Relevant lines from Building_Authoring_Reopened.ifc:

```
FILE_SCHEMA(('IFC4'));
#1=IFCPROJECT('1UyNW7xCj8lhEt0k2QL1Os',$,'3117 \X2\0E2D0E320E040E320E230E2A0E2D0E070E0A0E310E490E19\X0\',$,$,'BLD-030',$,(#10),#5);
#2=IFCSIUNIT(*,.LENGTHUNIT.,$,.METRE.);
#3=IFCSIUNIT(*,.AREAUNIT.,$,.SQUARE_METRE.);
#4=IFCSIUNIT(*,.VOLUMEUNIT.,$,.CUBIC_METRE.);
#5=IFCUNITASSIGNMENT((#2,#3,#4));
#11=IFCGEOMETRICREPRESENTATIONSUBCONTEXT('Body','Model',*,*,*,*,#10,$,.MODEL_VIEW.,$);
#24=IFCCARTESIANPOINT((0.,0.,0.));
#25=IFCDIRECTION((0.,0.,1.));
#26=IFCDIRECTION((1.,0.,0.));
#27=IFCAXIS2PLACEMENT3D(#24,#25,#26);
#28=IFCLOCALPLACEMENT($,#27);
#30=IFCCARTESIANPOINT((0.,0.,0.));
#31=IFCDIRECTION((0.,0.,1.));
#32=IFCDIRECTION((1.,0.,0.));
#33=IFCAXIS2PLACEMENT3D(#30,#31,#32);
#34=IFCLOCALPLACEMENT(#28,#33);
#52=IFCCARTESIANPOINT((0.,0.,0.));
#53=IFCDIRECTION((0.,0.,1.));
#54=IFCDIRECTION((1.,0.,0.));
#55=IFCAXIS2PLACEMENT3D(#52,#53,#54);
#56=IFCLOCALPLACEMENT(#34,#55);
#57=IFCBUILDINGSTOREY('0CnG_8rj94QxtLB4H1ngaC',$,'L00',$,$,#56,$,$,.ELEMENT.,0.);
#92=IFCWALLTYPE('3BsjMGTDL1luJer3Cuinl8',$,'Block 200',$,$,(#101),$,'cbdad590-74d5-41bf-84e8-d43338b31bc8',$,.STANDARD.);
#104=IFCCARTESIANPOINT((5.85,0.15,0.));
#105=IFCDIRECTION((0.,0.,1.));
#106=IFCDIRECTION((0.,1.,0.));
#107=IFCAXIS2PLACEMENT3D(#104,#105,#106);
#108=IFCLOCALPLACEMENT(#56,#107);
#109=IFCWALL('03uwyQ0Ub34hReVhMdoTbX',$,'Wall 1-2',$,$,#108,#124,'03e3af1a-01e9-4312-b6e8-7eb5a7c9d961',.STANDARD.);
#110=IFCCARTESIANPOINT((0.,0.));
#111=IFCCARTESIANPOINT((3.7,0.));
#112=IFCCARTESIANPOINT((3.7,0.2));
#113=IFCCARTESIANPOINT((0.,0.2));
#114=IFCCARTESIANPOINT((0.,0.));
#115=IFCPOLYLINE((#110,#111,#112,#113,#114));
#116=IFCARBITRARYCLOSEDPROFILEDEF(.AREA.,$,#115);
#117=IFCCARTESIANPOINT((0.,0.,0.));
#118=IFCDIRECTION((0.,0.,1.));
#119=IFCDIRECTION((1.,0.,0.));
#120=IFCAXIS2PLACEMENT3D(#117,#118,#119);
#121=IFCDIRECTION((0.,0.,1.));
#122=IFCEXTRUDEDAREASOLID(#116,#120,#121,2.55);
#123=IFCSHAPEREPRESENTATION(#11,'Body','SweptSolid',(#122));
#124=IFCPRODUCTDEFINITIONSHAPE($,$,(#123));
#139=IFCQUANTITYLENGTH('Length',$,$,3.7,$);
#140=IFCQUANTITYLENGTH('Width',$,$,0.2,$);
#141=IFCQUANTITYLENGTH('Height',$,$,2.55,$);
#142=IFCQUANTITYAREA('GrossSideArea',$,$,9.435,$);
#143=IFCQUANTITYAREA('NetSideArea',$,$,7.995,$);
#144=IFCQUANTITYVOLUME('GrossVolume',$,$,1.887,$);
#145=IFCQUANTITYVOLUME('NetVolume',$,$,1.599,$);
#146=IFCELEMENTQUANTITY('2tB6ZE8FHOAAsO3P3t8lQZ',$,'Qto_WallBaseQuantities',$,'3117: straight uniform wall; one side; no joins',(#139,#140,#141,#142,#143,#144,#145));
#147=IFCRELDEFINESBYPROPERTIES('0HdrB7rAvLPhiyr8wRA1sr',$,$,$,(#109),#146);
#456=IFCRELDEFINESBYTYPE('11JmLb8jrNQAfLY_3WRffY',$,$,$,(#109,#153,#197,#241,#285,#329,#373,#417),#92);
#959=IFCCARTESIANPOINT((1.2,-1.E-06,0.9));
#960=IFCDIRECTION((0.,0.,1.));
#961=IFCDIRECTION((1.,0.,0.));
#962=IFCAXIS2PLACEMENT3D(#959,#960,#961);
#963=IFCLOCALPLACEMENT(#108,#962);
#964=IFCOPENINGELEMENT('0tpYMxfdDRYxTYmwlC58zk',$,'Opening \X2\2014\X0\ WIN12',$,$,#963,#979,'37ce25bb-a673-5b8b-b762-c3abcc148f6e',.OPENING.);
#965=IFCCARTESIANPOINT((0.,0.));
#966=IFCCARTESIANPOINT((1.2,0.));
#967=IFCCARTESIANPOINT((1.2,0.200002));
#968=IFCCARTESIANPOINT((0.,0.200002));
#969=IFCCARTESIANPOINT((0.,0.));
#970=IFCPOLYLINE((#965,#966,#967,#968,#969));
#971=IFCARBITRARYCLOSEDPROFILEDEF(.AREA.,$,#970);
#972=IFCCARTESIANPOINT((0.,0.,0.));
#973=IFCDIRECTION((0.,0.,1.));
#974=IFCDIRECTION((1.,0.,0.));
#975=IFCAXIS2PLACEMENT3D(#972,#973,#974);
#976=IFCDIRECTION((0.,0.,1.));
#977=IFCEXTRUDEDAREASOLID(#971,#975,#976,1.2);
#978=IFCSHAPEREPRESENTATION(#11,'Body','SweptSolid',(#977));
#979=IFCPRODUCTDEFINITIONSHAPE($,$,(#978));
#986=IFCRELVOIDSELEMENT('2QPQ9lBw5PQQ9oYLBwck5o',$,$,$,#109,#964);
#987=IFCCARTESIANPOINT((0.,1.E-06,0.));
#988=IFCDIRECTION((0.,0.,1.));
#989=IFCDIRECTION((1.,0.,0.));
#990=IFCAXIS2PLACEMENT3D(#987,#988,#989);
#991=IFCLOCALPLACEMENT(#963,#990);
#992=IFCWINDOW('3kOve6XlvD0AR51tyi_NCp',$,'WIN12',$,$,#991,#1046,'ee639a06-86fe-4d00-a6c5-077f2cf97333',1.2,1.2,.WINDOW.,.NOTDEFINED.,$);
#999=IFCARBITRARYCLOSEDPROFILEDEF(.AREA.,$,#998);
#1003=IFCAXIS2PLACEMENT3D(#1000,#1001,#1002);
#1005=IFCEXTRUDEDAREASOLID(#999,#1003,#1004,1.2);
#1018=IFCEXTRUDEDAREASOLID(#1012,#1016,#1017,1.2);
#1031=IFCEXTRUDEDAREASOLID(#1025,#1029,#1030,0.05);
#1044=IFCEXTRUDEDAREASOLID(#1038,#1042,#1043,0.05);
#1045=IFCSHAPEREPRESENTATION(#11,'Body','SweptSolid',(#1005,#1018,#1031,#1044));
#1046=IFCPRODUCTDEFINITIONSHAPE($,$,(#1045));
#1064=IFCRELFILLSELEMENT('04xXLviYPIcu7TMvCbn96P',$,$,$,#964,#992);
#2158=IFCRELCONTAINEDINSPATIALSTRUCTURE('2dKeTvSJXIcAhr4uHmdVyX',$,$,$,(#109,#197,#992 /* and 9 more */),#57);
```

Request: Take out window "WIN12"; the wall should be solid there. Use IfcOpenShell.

```python
import ifcopenshell
import ifcopenshell.api.feature
import ifcopenshell.api.pset
import ifcopenshell.api.root
import ifcopenshell.geom
import ifcopenshell.util.element
import ifcopenshell.util.shape
import ifcopenshell.util.unit

model = ifcopenshell.open("Building_Authoring_Reopened.ifc")
area_scale = ifcopenshell.util.unit.calculate_unit_scale(model, "AREAUNIT")
volume_scale = ifcopenshell.util.unit.calculate_unit_scale(model, "VOLUMEUNIT")
settings = ifcopenshell.geom.settings()


def volume(element):
    """Net volume in cubic metres, openings subtracted."""
    shape = ifcopenshell.geom.create_shape(settings, element)
    return ifcopenshell.util.shape.get_volume(shape.geometry)


window = model.by_guid("3kOve6XlvD0AR51tyi_NCp")
opening = window.FillsVoids[0].RelatingOpeningElement
wall = opening.VoidsElements[0].RelatingBuildingElement
before = volume(wall)

ifcopenshell.api.root.remove_product(model, product=window)
ifcopenshell.api.feature.remove_feature(model, feature=opening)

after = volume(wall)
thickness = 0.2  # wall thickness in metres

# Update the wall's stored quantities.
qto = model.by_id(ifcopenshell.util.element.get_pset(wall, "Qto_WallBaseQuantities", should_inherit=False)["id"])
ifcopenshell.api.pset.edit_qto(model, qto=qto, properties={
    "NetSideArea": after / thickness / area_scale,
    "NetVolume": after / volume_scale,
})

print(f"wall volume {before:.3f} -> {after:.3f} m3")

model.write("Building_Authoring_Reopened_rev.ifc")
```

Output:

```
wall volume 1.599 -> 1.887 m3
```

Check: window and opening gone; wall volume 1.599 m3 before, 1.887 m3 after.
